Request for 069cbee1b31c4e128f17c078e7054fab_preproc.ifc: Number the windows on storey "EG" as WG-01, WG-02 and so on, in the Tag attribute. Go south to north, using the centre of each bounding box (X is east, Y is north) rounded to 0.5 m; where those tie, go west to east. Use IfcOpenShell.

First a look at what the model holds.

```python
import ifcopenshell
import ifcopenshell.util.element
import ifcopenshell.util.placement

model = ifcopenshell.open("069cbee1b31c4e128f17c078e7054fab_preproc.ifc")
print(model.schema)
storey = next(s for s in model.by_type("IfcBuildingStorey") if s.Name == "EG")
windows = [e for e in ifcopenshell.util.element.get_decomposition(storey) if e.is_a("IfcWindow")]
for e in sorted(windows, key=lambda e: e.id()):
    origin = ifcopenshell.util.placement.get_local_placement(e.ObjectPlacement)[:3, 3]
    print(e.id(), e.Tag, e.Name, origin.round(2) + 0.0, sep=" | ")
```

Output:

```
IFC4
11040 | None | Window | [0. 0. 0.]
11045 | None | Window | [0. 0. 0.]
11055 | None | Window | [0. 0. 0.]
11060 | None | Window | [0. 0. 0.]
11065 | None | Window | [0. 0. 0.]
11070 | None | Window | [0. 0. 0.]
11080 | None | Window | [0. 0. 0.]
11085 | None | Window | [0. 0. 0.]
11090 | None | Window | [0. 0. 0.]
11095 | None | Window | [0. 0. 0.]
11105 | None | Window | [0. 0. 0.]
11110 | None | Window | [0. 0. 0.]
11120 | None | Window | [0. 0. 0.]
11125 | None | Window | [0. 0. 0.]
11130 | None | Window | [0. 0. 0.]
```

```python
import ifcopenshell
import ifcopenshell.geom
import ifcopenshell.util.element
import ifcopenshell.util.shape

model = ifcopenshell.open("069cbee1b31c4e128f17c078e7054fab_preproc.ifc")
settings = ifcopenshell.geom.settings()
settings.set("use-world-coords", True)


def centre(element):
    shape = ifcopenshell.geom.create_shape(settings, element)
    return ifcopenshell.util.shape.get_bbox_centroid(shape.geometry)


storey = next(s for s in model.by_type("IfcBuildingStorey") if s.Name == "EG")
windows = [e for e in ifcopenshell.util.element.get_decomposition(storey) if e.is_a("IfcWindow")]

# Insertion points can sit at a corner or the storey origin, so sort by the geometry (in metres).
centres = {e: centre(e) for e in windows}
windows.sort(key=lambda e: (round(centres[e][1] / 0.5), centres[e][0]))

for i, e in enumerate(windows, start=1):
    number = f"WG-{i:02d}"
    e.Tag = number
    print(e.id(), number)

model.write("069cbee1b31c4e128f17c078e7054fab_preproc-out.ifc")
```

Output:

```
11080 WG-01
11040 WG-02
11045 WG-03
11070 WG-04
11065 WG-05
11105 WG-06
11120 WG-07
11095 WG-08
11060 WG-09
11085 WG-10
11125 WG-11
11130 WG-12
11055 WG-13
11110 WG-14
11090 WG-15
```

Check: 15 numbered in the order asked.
